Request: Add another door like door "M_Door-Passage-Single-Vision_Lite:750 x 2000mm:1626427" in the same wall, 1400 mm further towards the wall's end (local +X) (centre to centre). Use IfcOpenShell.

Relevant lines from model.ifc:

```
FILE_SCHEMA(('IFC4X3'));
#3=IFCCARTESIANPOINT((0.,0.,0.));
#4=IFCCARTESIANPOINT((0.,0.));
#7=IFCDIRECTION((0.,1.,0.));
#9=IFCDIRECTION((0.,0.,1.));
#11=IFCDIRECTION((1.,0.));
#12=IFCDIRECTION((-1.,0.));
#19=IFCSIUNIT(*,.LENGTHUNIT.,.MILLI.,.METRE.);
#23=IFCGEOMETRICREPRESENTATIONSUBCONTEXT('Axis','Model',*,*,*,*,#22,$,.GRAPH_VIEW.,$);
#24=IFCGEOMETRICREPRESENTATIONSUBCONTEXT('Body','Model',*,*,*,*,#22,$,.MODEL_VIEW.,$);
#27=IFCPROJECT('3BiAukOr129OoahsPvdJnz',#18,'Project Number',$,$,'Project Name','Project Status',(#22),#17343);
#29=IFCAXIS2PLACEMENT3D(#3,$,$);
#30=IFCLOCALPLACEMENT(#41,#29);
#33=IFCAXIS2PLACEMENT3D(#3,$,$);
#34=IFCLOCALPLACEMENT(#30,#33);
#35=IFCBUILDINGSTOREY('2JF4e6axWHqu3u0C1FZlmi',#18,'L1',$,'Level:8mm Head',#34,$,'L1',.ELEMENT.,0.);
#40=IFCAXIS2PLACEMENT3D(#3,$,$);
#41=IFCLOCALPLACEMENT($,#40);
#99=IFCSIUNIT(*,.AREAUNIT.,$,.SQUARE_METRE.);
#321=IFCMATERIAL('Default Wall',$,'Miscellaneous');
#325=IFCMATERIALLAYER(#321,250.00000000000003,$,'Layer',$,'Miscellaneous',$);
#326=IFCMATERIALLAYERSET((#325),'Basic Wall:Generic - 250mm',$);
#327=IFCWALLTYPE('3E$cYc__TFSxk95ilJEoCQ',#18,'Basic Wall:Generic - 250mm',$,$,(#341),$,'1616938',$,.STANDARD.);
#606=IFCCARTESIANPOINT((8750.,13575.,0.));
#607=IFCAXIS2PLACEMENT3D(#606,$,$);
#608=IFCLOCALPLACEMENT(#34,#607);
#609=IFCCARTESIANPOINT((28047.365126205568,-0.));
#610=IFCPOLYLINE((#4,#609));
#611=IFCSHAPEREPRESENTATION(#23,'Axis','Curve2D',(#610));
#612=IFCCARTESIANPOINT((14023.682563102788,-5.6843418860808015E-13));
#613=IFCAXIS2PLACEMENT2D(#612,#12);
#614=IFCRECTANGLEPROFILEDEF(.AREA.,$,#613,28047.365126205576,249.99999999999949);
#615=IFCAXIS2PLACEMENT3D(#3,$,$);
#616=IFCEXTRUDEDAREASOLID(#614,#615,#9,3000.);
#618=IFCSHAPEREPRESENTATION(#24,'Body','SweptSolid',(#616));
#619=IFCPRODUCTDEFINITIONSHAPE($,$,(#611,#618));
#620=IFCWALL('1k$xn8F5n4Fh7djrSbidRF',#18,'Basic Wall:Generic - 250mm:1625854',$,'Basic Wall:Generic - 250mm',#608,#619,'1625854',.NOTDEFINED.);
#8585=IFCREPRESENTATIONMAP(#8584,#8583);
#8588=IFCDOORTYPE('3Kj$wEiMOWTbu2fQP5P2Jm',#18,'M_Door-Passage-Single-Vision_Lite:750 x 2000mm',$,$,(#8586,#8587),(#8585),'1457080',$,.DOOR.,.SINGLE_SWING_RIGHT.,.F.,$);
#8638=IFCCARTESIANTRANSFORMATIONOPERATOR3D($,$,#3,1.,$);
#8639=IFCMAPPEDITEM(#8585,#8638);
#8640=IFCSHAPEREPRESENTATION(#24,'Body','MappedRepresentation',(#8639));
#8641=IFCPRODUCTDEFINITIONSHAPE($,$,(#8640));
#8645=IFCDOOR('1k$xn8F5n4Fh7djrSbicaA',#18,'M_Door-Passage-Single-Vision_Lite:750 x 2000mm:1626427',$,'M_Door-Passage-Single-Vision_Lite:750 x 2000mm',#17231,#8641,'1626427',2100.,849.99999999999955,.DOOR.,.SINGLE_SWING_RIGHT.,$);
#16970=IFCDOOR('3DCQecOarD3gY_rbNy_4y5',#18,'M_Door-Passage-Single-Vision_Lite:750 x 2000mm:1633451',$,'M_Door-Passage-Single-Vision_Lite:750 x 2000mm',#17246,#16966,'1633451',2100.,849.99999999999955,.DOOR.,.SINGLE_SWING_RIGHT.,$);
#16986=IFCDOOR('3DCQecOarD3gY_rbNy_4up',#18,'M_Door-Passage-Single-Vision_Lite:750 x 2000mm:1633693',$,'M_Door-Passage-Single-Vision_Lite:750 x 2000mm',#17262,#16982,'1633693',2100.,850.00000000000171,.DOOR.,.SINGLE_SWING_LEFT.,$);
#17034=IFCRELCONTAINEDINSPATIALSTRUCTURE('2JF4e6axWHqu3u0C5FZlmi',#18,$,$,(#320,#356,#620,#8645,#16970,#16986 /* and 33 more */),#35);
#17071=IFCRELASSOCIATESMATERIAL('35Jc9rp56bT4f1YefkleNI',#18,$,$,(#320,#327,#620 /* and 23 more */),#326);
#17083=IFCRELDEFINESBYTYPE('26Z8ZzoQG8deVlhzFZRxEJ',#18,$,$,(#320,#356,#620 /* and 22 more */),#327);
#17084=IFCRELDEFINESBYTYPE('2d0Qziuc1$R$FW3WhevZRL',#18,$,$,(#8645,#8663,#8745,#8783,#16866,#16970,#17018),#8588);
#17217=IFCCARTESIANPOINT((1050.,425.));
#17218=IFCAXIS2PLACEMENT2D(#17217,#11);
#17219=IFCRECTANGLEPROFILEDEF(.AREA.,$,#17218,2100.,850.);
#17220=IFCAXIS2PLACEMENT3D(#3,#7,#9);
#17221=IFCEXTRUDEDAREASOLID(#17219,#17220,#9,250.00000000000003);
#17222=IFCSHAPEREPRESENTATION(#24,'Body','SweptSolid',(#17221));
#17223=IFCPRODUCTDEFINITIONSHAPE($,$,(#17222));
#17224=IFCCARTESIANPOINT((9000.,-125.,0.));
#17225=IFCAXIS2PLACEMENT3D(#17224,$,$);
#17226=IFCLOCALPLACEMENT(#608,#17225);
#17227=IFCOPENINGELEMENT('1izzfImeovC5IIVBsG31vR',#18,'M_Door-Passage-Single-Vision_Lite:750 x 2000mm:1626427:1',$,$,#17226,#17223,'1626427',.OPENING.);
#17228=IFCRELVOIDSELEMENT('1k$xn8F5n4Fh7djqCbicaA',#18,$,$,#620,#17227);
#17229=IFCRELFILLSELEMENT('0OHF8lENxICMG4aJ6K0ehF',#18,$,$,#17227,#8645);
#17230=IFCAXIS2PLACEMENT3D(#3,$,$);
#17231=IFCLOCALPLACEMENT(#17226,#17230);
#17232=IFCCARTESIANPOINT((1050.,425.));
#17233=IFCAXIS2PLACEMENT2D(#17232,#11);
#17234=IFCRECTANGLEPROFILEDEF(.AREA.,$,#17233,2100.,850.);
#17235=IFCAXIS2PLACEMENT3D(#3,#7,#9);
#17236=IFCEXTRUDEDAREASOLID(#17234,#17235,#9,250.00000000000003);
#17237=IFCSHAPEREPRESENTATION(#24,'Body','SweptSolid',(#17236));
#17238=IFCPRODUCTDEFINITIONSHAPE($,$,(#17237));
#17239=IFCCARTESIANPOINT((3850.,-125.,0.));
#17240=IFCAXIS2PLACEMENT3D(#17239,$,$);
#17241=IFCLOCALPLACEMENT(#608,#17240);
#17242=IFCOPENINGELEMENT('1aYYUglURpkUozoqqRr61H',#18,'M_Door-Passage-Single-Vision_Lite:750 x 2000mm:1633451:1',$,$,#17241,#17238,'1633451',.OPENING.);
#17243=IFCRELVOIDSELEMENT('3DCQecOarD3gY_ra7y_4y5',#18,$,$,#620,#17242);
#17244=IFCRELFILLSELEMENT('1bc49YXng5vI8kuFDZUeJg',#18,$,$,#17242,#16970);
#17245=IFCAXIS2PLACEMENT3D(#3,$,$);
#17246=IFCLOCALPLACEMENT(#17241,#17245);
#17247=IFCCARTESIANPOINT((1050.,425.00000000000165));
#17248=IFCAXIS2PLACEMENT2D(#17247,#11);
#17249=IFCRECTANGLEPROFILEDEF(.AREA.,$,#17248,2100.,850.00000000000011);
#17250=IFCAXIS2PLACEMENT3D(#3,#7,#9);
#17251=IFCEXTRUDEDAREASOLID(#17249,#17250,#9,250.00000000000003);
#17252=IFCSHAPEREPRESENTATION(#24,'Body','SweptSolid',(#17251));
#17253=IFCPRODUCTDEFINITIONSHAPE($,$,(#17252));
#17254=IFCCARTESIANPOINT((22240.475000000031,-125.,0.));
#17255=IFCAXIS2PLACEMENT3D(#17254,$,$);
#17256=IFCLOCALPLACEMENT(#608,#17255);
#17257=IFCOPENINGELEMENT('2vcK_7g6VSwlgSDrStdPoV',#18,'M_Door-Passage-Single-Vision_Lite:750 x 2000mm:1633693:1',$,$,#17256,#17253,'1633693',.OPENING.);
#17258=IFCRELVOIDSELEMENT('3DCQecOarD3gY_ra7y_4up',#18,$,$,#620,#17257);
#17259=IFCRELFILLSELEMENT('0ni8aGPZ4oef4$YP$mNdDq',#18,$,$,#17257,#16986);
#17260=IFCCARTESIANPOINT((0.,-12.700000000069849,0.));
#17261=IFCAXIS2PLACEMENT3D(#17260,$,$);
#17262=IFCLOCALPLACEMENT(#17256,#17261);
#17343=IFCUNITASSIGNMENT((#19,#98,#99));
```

```python
import ifcopenshell
import ifcopenshell.api.feature
import ifcopenshell.api.geometry
import ifcopenshell.api.root
import ifcopenshell.geom
import ifcopenshell.util.element
import ifcopenshell.util.placement
import ifcopenshell.util.shape
import ifcopenshell.util.unit

model = ifcopenshell.open("model.ifc")
unit_scale = ifcopenshell.util.unit.calculate_unit_scale(model)
settings = ifcopenshell.geom.settings()


def volume(element):
    """Net volume in cubic metres, openings subtracted."""
    shape = ifcopenshell.geom.create_shape(settings, element)
    return ifcopenshell.util.shape.get_volume(shape.geometry)


def reuse_history(source, copy):
    """copy_class also copies each property set's owner history, people and application; keep the originals."""
    for rel in copy.IsDefinedBy:
        if rel.is_a("IfcRelDefinesByProperties") and (history := rel.RelatingPropertyDefinition.OwnerHistory):
            rel.RelatingPropertyDefinition.OwnerHistory = source.OwnerHistory
            ifcopenshell.util.element.remove_deep2(model, history)


door = model.by_guid("1k$xn8F5n4Fh7djrSbicaA")
opening = door.FillsVoids[0].RelatingOpeningElement
wall = opening.VoidsElements[0].RelatingBuildingElement
before = volume(wall)
shift = ifcopenshell.util.placement.get_local_placement(wall.ObjectPlacement)[:3, 0] * 1.4 / unit_scale

# copy_class copies the void relationship, type, container and properties, but no geometry.
new_opening = ifcopenshell.api.root.copy_class(model, product=opening)
new_opening.Representation = ifcopenshell.util.element.copy_deep(
    model, opening.Representation, exclude=["IfcGeometricRepresentationContext", "IfcRepresentationMap"]
)
new_opening.Name = "M_Door-Passage-Single-Vision_Lite:750 x 2000mm"
new_opening.Tag = None
new_door = ifcopenshell.api.root.copy_class(model, product=door)
new_door.Representation = ifcopenshell.util.element.copy_deep(
    model, door.Representation, exclude=["IfcGeometricRepresentationContext", "IfcRepresentationMap"]
)
new_door.Name = "M_Door-Passage-Single-Vision_Lite:750 x 2000mm"
new_door.Tag = None
reuse_history(door, new_door)
ifcopenshell.api.feature.add_filling(model, opening=new_opening, element=new_door)

for old, new in ((opening, new_opening), (door, new_door)):
    matrix = ifcopenshell.util.placement.get_local_placement(old.ObjectPlacement)
    matrix[:3, 3] += shift
    ifcopenshell.api.geometry.edit_object_placement(model, product=new, matrix=matrix, is_si=False)

after = volume(wall)

print(f"wall volume {before:.3f} -> {after:.3f} m3")

model.write("model-out.ifc")
```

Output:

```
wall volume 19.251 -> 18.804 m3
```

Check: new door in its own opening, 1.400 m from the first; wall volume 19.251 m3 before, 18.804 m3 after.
